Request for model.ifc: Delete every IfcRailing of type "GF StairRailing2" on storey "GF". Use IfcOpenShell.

First a look at what the model holds.

```python
import ifcopenshell
import ifcopenshell.util.element

model = ifcopenshell.open("model.ifc")
print(model.schema)
storey = next(s for s in model.by_type("IfcBuildingStorey") if s.Name == "GF")
railings = [e for e in ifcopenshell.util.element.get_decomposition(storey) if e.is_a("IfcRailing")]
seen = {}
for e in railings:
    element_type = ifcopenshell.util.element.get_type(e)
    name = element_type.Name if element_type not in (None, e) else None
    seen[name] = seen.get(name, 0) + 1
for name, count in sorted(seen.items(), key=str):
    print(count, "x", name)
```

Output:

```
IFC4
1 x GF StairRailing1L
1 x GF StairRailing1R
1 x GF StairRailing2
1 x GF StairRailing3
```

```python
import ifcopenshell
import ifcopenshell.api.root
import ifcopenshell.util.element

model = ifcopenshell.open("model.ifc")

storey = next(s for s in model.by_type("IfcBuildingStorey") if s.Name == "GF")
railings = [e for e in ifcopenshell.util.element.get_decomposition(storey) if e.is_a("IfcRailing")]
targets = [e for e in railings if (t := ifcopenshell.util.element.get_type(e)) not in (None, e) and t.Name == "GF StairRailing2"]

for e in targets:
    ifcopenshell.api.root.remove_product(model, product=e)
print(len(targets), "removed")

model.write("model_rev.ifc")
```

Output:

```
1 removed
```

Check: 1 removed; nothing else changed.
